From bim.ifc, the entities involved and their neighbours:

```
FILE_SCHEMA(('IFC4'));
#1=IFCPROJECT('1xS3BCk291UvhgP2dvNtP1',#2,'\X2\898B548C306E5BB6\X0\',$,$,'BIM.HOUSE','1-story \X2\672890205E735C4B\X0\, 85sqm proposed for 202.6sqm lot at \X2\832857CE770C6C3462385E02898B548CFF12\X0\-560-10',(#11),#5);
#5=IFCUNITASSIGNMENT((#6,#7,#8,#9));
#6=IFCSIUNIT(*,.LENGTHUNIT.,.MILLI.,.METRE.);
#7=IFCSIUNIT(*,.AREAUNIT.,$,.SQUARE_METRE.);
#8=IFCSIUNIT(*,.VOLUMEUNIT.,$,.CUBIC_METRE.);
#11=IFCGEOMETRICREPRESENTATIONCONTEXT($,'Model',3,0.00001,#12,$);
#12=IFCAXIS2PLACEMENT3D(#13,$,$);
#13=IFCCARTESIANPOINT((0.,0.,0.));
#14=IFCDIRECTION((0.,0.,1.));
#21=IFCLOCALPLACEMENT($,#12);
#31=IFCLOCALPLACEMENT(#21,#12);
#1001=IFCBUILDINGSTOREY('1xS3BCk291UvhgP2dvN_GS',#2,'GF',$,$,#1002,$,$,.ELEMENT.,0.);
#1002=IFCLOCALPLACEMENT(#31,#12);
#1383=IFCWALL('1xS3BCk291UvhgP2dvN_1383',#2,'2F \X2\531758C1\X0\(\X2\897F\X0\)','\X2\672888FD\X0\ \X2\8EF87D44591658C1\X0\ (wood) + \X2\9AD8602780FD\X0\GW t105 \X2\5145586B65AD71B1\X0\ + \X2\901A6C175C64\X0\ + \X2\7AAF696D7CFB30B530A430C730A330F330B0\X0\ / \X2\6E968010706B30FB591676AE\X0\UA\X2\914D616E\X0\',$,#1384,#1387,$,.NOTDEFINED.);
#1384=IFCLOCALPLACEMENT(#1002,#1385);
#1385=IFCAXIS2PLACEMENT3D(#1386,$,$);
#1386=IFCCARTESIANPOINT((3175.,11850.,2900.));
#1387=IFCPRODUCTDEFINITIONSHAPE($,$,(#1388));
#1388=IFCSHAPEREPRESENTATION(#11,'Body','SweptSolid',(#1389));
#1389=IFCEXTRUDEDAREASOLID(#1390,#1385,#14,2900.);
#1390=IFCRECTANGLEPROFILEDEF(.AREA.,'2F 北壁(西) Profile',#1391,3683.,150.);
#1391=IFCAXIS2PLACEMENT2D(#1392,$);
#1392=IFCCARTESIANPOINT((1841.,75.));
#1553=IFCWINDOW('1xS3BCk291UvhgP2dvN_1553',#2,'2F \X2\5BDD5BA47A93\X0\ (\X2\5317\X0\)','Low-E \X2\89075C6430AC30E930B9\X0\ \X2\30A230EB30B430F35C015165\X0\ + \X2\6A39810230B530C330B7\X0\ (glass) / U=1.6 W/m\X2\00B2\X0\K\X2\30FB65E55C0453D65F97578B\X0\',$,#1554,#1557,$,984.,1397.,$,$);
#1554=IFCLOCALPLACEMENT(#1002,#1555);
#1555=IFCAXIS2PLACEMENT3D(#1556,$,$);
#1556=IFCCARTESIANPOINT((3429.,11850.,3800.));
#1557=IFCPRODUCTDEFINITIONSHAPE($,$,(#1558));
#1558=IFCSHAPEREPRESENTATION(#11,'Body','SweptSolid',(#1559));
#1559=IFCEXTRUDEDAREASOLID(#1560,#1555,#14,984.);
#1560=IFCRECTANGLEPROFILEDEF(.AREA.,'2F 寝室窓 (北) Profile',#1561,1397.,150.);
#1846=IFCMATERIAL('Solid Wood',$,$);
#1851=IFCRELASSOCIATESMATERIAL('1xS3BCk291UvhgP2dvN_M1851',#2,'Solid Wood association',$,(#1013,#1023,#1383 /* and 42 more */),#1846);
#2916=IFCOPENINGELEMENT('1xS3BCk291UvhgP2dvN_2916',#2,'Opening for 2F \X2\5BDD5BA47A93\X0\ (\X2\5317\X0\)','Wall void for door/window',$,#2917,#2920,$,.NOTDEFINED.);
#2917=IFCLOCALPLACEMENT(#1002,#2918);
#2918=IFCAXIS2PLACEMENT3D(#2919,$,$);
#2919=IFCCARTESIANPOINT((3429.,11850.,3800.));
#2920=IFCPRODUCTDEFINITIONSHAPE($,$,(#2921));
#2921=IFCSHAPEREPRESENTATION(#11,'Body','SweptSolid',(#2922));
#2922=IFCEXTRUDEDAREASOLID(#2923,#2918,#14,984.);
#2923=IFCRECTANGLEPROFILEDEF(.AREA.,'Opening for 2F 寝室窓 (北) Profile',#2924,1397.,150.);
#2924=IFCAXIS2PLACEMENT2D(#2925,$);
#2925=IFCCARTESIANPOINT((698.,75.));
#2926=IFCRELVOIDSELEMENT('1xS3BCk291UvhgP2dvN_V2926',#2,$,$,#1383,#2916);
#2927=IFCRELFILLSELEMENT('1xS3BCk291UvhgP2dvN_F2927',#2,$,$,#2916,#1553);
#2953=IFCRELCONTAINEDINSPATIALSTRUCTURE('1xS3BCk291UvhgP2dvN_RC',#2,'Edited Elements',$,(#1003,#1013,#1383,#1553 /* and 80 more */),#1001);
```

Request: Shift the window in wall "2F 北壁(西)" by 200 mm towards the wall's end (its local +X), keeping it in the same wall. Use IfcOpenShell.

```python
import ifcopenshell
import ifcopenshell.api.geometry
import ifcopenshell.util.placement
import ifcopenshell.util.unit

model = ifcopenshell.open("bim.ifc")
unit_scale = ifcopenshell.util.unit.calculate_unit_scale(model)

window = model.by_guid("1xS3BCk291UvhgP2dvN_1553")
opening = window.FillsVoids[0].RelatingOpeningElement
wall = opening.VoidsElements[0].RelatingBuildingElement

wall_matrix = ifcopenshell.util.placement.get_local_placement(wall.ObjectPlacement)
shift = wall_matrix[:3, 0] * 0.2 / unit_scale
before = ifcopenshell.util.placement.get_local_placement(window.ObjectPlacement)[:3, 3].copy()

# The window is not placed relative to its opening, so move both.
for product in (opening, window):
    matrix = ifcopenshell.util.placement.get_local_placement(product.ObjectPlacement)
    matrix[:3, 3] += shift
    ifcopenshell.api.geometry.edit_object_placement(model, product=product, matrix=matrix, is_si=False)

after = ifcopenshell.util.placement.get_local_placement(window.ObjectPlacement)[:3, 3]
print("window moved by", (after - before).round(3) + 0.0)

model.write("bim_updated.ifc")
```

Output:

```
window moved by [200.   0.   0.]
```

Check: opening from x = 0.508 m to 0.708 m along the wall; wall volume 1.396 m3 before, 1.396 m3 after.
